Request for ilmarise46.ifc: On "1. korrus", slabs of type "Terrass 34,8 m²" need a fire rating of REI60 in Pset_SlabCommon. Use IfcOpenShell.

First a look at what the model holds.

```python
import ifcopenshell
import ifcopenshell.util.element

model = ifcopenshell.open("ilmarise46.ifc")
print(model.schema)
storey = next(s for s in model.by_type("IfcBuildingStorey") if s.Name == "1. korrus")
slabs = [e for e in ifcopenshell.util.element.get_decomposition(storey) if e.is_a("IfcSlab")]
seen = {}
for e in slabs:
    element_type = ifcopenshell.util.element.get_type(e)
    key = (element_type.Name if element_type != e and element_type else None, ifcopenshell.util.element.get_pset(e, "Pset_SlabCommon", "FireRating"))
    seen[key] = seen.get(key, 0) + 1
for (name, value), count in sorted(seen.items(), key=str):
    print(count, "x", name, "|", value)
```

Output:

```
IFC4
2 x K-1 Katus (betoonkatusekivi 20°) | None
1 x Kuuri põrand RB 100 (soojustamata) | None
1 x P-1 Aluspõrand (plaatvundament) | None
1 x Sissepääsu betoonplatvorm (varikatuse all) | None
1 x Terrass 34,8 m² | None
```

```python
import ifcopenshell
import ifcopenshell.api.pset
import ifcopenshell.util.element

model = ifcopenshell.open("ilmarise46.ifc")

storey = next(s for s in model.by_type("IfcBuildingStorey") if s.Name == "1. korrus")
slabs = [e for e in ifcopenshell.util.element.get_decomposition(storey) if e.is_a("IfcSlab")]

count = 0
for e in slabs:
    element_type = ifcopenshell.util.element.get_type(e)
    if element_type in (None, e) or element_type.Name != "Terrass 34,8 m²":
        continue
    # add_pset returns the element's existing set when there is one.
    pset = ifcopenshell.api.pset.add_pset(model, product=e, name="Pset_SlabCommon")
    ifcopenshell.api.pset.edit_pset(model, pset=pset, properties={"FireRating": "REI60"})
    count += 1

print(count, "slabs updated")

model.write("ilmarise46_edited.ifc")
```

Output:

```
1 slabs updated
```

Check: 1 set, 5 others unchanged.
